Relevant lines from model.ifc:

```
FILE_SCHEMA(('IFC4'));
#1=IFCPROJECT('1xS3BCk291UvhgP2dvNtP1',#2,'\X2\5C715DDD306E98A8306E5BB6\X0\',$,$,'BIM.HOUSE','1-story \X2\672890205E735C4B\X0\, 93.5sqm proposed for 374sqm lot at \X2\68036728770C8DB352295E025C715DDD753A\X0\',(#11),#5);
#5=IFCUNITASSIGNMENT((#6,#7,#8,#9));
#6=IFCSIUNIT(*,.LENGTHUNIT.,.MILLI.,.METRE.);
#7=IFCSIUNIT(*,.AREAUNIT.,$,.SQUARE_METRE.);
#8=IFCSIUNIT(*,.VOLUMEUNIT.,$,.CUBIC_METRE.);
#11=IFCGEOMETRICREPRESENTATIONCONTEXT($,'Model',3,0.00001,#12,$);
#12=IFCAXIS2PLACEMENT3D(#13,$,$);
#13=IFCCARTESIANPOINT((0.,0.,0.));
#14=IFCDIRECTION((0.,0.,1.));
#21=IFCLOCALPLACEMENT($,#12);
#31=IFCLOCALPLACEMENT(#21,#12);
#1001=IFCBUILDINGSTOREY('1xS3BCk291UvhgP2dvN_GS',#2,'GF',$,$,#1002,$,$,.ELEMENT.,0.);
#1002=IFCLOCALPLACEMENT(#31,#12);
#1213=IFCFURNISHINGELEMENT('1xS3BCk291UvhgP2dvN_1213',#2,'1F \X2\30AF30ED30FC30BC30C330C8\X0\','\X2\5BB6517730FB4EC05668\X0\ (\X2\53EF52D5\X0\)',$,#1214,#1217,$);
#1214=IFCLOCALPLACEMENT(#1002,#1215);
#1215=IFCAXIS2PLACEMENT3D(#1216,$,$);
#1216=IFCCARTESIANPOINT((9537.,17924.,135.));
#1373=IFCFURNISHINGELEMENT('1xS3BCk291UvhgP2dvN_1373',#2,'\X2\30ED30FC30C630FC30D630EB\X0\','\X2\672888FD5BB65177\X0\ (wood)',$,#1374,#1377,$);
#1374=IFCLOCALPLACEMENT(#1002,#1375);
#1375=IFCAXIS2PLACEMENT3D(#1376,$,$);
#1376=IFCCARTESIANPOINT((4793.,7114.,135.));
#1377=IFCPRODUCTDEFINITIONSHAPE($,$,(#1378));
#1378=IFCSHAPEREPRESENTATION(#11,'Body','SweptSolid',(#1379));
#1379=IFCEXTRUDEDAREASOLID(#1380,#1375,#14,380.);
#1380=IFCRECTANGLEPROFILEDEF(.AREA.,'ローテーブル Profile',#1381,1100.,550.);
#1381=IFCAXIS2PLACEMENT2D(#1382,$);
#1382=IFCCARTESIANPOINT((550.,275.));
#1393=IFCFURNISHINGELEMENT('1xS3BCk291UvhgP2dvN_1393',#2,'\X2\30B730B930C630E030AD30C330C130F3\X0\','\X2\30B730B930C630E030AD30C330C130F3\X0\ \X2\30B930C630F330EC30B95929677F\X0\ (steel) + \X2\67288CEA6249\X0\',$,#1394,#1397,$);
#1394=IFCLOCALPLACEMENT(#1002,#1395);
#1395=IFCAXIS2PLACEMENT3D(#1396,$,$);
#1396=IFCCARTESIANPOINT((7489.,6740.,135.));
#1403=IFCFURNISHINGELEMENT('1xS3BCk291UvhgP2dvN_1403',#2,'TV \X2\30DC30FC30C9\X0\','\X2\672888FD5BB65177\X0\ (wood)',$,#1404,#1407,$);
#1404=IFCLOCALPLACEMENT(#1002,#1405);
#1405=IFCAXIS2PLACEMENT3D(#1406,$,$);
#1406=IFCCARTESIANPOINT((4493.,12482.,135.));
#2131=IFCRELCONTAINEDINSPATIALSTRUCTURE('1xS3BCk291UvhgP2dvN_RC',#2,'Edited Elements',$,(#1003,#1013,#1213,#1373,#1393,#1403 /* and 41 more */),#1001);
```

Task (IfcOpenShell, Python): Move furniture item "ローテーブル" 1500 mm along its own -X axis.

```python
import ifcopenshell
import ifcopenshell.api.geometry
import ifcopenshell.util.placement

model = ifcopenshell.open("model.ifc")

item = model.by_guid("1xS3BCk291UvhgP2dvN_1373")
matrix = ifcopenshell.util.placement.get_local_placement(item.ObjectPlacement)
matrix[:3, 3] -= matrix[:3, 0] * 1500.0
ifcopenshell.api.geometry.edit_object_placement(model, product=item, matrix=matrix, is_si=False)

print(ifcopenshell.util.placement.get_local_placement(item.ObjectPlacement).round(3) + 0.0)

model.write("model_edited.ifc")
```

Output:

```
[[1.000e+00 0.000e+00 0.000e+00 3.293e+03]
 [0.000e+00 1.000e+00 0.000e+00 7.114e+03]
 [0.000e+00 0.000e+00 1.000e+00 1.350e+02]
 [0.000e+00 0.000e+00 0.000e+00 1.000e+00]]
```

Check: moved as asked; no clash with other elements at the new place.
